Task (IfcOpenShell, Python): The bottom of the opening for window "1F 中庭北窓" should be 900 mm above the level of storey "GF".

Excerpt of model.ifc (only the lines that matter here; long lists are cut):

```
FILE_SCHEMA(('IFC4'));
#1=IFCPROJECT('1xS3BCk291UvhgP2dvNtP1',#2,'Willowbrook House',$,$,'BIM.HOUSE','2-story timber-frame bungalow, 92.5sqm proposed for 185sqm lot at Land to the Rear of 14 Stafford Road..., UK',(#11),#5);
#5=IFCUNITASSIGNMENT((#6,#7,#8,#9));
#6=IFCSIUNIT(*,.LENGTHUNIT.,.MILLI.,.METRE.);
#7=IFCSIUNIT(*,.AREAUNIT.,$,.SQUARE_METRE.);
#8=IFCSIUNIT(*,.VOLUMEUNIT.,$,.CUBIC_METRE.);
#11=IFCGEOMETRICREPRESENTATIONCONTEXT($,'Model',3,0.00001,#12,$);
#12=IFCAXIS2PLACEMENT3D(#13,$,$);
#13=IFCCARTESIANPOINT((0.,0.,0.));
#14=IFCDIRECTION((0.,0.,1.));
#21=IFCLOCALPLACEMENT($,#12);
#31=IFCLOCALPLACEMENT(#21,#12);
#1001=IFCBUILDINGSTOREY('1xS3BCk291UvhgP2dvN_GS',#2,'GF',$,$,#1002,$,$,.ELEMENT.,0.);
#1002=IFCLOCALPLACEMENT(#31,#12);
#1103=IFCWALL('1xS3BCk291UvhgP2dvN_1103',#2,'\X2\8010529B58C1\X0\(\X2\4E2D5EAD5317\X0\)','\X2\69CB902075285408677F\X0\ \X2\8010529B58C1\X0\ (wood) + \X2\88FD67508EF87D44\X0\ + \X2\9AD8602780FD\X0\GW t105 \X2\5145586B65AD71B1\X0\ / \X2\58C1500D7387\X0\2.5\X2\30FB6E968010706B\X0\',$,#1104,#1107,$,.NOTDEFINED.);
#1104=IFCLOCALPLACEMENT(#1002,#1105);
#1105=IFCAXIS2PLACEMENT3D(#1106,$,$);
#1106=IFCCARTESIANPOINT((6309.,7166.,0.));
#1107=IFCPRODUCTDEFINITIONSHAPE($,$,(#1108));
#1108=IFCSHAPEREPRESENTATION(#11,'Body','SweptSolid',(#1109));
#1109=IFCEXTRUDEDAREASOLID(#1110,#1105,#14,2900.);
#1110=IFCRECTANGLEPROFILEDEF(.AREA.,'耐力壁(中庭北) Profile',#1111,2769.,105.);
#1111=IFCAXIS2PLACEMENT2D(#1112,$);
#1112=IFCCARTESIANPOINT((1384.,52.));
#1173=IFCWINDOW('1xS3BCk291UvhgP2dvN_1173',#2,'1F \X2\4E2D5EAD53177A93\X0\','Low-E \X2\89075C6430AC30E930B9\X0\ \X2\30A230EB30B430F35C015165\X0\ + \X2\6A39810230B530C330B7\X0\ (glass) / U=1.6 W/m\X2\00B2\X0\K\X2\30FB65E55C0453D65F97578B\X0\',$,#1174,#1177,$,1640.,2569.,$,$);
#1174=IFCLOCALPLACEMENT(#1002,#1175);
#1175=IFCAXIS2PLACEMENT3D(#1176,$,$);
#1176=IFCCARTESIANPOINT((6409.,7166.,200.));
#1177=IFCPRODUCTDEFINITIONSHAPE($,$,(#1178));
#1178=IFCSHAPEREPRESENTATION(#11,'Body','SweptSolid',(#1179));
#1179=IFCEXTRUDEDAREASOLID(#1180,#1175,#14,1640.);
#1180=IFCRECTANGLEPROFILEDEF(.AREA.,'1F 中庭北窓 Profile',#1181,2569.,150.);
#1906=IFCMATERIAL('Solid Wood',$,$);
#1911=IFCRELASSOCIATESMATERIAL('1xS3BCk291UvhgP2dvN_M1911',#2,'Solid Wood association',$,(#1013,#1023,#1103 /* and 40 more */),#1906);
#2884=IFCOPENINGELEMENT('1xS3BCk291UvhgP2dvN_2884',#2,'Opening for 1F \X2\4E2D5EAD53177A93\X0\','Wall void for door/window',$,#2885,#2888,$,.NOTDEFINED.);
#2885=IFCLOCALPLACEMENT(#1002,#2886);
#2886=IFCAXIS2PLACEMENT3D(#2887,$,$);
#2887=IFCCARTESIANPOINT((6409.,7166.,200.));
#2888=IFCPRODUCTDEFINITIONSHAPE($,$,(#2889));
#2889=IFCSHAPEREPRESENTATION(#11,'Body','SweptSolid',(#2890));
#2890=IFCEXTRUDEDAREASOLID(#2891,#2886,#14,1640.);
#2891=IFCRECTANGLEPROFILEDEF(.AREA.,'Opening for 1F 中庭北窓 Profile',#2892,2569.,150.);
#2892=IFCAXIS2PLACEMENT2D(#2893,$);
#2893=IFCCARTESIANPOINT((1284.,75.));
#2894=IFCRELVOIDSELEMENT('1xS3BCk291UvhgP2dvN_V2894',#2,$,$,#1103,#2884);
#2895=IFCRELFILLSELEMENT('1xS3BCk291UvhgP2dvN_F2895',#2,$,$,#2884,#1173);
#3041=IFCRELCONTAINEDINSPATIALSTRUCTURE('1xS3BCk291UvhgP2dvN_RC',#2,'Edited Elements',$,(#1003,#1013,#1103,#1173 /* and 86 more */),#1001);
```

```python
import numpy as np
import ifcopenshell
import ifcopenshell.api.geometry
import ifcopenshell.geom
import ifcopenshell.util.element
import ifcopenshell.util.placement
import ifcopenshell.util.shape
import ifcopenshell.util.unit

model = ifcopenshell.open("model.ifc")
unit_scale = ifcopenshell.util.unit.calculate_unit_scale(model)

window = model.by_id(1173)
opening = window.FillsVoids[0].RelatingOpeningElement
storey = ifcopenshell.util.element.get_container(window, ifc_class="IfcBuildingStorey")
level = ifcopenshell.util.placement.get_local_placement(storey.ObjectPlacement)[2, 3]

# The opening's origin need not be at the sill, so measure its lowest point.
shape = ifcopenshell.geom.create_shape(ifcopenshell.geom.settings(), opening)
bottom = ifcopenshell.util.shape.get_shape_bottom_elevation(shape, shape.geometry) / unit_scale
dz = level + 0.9 / unit_scale - bottom

shift = np.array([0.0, 0.0, dz])
# The window is not placed relative to its opening, so move both.
for product in (opening, window):
    matrix = ifcopenshell.util.placement.get_local_placement(product.ObjectPlacement)
    matrix[:3, 3] += shift
    ifcopenshell.api.geometry.edit_object_placement(model, product=product, matrix=matrix, is_si=False)

print(f"moved by {dz * unit_scale:+.3f} m")

model.write("model_edited.ifc")
```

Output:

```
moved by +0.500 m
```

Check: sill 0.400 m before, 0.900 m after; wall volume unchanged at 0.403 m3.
